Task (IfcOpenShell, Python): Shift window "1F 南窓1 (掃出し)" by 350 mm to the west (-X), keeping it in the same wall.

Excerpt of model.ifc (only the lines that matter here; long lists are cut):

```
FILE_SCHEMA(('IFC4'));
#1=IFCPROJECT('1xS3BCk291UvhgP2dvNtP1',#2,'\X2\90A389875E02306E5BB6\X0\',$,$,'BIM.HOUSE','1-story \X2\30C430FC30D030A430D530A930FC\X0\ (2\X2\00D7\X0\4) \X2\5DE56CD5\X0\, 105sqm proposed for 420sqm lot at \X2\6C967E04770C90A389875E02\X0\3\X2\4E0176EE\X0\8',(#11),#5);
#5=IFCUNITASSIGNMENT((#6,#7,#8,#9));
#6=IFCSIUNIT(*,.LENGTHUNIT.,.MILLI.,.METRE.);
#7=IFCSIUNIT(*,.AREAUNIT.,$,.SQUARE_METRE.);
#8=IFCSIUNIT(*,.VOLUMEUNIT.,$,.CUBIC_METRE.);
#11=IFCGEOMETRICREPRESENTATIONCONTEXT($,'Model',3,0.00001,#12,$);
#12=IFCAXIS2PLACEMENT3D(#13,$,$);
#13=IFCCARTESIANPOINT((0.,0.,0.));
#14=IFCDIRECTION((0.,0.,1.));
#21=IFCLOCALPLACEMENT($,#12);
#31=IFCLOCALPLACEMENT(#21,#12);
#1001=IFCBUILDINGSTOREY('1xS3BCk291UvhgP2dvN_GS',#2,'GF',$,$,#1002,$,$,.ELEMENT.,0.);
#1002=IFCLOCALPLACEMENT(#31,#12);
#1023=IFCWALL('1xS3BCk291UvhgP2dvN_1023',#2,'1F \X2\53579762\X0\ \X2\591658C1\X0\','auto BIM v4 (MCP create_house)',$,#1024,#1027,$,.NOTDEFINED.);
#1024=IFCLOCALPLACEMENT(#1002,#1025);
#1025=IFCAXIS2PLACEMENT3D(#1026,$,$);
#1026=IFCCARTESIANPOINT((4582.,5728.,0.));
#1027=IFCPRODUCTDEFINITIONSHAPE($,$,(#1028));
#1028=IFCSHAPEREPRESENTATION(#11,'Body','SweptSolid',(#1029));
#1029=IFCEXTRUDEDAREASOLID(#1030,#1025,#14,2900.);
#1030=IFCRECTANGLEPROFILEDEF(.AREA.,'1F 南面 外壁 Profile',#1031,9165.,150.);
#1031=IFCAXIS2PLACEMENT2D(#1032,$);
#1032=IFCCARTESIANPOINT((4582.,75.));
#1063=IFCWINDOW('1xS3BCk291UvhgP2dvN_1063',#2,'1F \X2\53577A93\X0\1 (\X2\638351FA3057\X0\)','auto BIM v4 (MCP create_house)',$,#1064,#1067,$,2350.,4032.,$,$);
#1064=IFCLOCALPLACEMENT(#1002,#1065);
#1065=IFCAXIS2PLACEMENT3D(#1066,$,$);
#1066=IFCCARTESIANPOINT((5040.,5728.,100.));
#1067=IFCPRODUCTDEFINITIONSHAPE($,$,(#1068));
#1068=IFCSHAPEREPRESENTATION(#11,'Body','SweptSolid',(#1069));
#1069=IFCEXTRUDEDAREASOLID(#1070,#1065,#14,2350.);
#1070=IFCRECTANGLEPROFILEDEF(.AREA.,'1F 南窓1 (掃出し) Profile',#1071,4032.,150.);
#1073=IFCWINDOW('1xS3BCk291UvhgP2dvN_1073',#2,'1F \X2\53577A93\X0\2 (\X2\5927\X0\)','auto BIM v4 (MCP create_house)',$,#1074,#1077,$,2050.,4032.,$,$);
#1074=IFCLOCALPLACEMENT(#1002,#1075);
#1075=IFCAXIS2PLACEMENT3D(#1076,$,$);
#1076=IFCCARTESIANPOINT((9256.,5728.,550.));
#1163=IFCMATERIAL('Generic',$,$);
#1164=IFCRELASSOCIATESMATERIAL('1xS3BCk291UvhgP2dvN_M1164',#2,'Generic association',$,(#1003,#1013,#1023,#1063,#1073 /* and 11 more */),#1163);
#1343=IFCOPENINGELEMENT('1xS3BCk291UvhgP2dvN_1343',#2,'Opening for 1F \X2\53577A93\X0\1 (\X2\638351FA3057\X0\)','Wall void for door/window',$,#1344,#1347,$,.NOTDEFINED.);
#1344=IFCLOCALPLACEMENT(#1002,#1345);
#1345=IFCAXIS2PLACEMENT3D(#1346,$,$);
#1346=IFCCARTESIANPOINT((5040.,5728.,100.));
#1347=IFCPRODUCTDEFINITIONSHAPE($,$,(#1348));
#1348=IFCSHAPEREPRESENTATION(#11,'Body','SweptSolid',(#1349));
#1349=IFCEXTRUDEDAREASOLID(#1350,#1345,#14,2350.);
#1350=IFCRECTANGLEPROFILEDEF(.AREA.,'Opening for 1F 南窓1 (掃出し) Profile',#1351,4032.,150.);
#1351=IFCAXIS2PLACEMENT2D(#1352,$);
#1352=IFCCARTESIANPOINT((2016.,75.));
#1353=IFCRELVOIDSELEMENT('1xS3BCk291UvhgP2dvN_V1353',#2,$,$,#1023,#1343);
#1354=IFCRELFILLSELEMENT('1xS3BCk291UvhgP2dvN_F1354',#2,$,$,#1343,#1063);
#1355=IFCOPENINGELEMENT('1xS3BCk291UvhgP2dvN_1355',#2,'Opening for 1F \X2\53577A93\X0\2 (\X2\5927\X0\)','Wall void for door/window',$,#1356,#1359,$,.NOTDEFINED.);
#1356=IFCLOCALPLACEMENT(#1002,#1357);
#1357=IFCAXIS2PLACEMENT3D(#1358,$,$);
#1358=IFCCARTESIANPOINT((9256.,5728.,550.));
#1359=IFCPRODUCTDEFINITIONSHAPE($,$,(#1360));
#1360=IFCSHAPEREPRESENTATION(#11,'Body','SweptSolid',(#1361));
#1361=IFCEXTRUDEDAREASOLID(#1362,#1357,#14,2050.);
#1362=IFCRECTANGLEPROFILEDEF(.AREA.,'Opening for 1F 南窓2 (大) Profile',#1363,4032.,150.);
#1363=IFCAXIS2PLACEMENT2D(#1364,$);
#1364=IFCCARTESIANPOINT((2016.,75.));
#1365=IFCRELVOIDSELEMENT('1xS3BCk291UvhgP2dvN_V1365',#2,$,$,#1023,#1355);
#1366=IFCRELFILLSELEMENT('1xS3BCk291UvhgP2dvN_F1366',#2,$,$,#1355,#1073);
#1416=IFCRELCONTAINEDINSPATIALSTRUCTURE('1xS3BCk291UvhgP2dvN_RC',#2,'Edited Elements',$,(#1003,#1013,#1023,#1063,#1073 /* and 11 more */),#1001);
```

```python
import ifcopenshell
import ifcopenshell.api.geometry
import ifcopenshell.util.placement
import ifcopenshell.util.unit

model = ifcopenshell.open("model.ifc")
unit_scale = ifcopenshell.util.unit.calculate_unit_scale(model)

window = model.by_id(1063)
opening = window.FillsVoids[0].RelatingOpeningElement
wall = opening.VoidsElements[0].RelatingBuildingElement

wall_matrix = ifcopenshell.util.placement.get_local_placement(wall.ObjectPlacement)
shift = wall_matrix[:3, 0] * -0.35 / unit_scale
before = ifcopenshell.util.placement.get_local_placement(window.ObjectPlacement)[:3, 3].copy()

# The window is not placed relative to its opening, so move both.
for product in (opening, window):
    matrix = ifcopenshell.util.placement.get_local_placement(product.ObjectPlacement)
    matrix[:3, 3] += shift
    ifcopenshell.api.geometry.edit_object_placement(model, product=product, matrix=matrix, is_si=False)

after = ifcopenshell.util.placement.get_local_placement(window.ObjectPlacement)[:3, 3]
print("window moved by", (after - before).round(3) + 0.0)

model.write("model-out.ifc")
```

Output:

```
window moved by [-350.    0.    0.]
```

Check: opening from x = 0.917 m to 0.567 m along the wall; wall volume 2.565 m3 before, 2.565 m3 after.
